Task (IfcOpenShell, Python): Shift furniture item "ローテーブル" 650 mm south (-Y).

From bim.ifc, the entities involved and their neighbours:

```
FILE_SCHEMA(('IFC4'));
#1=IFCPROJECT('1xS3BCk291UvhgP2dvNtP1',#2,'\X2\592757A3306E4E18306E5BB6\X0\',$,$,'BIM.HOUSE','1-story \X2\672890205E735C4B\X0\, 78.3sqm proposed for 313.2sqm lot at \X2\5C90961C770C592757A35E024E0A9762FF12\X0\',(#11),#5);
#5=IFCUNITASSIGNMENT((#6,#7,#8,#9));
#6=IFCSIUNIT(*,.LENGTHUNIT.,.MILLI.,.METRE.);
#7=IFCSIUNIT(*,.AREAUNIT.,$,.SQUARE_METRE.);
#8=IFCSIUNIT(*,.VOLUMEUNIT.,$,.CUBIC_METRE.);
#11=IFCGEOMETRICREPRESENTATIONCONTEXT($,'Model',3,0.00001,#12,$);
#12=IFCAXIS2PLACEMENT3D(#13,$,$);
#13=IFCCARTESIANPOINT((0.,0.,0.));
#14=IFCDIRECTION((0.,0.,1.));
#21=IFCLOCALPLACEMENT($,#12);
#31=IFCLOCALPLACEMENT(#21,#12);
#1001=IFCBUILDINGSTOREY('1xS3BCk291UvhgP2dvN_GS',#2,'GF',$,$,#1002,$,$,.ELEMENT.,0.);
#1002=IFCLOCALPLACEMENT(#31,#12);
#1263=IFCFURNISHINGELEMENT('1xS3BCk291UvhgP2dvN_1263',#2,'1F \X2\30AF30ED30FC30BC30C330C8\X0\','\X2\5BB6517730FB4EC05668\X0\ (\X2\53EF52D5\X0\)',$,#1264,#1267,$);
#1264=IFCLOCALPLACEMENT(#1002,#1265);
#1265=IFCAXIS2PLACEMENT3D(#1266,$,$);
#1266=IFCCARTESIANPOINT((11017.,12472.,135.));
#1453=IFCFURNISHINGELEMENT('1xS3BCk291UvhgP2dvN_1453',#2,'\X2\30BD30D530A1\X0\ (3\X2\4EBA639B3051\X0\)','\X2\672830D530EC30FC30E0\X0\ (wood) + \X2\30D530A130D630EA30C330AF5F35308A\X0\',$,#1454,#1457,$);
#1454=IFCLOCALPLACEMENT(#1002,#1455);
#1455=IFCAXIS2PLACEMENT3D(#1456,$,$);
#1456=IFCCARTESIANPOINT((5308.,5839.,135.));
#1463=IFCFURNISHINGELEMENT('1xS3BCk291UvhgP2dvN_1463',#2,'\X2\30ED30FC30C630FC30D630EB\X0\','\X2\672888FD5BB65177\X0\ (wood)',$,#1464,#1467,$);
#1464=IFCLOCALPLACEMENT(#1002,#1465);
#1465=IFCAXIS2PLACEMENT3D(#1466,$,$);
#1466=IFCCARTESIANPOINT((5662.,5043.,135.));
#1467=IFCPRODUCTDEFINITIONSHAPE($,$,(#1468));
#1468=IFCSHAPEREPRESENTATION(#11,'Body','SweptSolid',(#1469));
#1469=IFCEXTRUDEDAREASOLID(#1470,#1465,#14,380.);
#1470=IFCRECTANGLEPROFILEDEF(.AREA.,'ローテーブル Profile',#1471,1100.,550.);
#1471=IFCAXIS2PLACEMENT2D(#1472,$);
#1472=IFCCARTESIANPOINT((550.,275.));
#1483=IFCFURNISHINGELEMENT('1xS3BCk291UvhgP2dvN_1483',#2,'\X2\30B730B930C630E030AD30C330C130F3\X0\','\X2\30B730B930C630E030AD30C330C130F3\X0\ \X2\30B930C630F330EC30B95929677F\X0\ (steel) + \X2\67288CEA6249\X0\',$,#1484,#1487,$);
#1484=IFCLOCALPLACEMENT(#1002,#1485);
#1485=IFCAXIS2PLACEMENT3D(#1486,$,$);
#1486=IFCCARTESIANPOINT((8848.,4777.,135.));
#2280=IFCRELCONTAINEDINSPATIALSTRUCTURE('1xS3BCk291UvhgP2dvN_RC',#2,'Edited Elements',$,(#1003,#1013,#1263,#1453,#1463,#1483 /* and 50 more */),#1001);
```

```python
import ifcopenshell
import ifcopenshell.api.geometry
import ifcopenshell.util.placement
import ifcopenshell.util.unit

model = ifcopenshell.open("bim.ifc")
unit_scale = ifcopenshell.util.unit.calculate_unit_scale(model)

item = model.by_guid("1xS3BCk291UvhgP2dvN_1463")
matrix = ifcopenshell.util.placement.get_local_placement(item.ObjectPlacement)
matrix[1, 3] -= 0.65 / unit_scale
ifcopenshell.api.geometry.edit_object_placement(model, product=item, matrix=matrix, is_si=False)

print(ifcopenshell.util.placement.get_local_placement(item.ObjectPlacement).round(3) + 0.0)

model.write("bim_v2.ifc")
```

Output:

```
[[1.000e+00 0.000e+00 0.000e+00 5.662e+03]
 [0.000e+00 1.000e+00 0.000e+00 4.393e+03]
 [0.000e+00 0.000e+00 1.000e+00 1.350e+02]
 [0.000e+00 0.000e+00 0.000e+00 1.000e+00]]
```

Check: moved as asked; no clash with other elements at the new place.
